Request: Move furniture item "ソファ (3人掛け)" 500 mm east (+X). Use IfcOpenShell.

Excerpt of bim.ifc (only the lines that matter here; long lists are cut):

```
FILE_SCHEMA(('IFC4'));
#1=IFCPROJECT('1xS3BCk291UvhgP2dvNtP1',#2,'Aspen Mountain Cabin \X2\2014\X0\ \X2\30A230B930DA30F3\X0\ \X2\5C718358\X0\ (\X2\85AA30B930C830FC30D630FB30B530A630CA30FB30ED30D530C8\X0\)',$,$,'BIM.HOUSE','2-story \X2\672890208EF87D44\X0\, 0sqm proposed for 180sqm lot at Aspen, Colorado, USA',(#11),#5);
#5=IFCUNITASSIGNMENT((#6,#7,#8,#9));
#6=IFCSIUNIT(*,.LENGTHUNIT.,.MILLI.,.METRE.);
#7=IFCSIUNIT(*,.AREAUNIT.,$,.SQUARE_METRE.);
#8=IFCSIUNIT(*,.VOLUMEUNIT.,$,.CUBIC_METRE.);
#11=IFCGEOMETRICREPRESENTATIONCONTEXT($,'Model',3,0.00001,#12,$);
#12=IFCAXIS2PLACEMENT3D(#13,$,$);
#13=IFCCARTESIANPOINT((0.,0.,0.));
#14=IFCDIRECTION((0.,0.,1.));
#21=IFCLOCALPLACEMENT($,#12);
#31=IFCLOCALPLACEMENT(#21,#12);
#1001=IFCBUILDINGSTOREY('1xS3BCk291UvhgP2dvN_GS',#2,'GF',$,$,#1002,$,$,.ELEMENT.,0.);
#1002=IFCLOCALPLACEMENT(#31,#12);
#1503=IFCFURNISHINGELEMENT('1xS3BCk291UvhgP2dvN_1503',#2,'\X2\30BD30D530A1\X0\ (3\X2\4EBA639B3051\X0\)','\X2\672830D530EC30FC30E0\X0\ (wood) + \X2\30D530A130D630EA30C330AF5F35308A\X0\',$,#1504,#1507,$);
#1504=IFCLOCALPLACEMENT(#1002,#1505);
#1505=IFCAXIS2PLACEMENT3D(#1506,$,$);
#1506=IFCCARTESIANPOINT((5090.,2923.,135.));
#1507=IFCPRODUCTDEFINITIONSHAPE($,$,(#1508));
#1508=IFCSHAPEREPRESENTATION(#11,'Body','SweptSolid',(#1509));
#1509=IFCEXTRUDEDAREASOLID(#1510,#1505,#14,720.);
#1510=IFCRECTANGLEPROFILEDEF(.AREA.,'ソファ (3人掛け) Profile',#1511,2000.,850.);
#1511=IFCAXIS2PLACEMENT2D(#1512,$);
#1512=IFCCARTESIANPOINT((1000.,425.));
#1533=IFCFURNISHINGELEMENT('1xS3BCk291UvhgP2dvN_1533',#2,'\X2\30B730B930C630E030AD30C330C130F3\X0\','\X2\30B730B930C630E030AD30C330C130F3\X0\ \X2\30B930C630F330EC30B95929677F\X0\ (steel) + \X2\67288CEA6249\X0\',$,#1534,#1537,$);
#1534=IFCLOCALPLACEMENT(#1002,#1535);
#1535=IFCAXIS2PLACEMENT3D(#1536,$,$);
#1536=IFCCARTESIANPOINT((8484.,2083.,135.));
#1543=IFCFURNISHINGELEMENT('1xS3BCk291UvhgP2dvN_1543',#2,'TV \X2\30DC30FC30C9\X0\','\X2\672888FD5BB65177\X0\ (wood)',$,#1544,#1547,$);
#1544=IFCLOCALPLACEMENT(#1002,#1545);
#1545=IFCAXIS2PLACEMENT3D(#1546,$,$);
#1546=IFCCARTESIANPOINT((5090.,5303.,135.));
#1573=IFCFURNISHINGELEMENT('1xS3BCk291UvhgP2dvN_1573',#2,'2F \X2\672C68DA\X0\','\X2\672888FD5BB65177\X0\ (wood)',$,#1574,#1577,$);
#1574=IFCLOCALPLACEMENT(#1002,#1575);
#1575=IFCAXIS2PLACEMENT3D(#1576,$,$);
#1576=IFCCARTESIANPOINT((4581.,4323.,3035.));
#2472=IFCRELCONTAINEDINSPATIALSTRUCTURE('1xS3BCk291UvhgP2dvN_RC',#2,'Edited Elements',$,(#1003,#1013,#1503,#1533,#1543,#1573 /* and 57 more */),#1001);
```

```python
import ifcopenshell
import ifcopenshell.api.geometry
import ifcopenshell.util.placement
import ifcopenshell.util.unit

model = ifcopenshell.open("bim.ifc")
unit_scale = ifcopenshell.util.unit.calculate_unit_scale(model)

item = model.by_guid("1xS3BCk291UvhgP2dvN_1503")
matrix = ifcopenshell.util.placement.get_local_placement(item.ObjectPlacement)
matrix[0, 3] += 0.5 / unit_scale
ifcopenshell.api.geometry.edit_object_placement(model, product=item, matrix=matrix, is_si=False)

print(ifcopenshell.util.placement.get_local_placement(item.ObjectPlacement).round(3) + 0.0)

model.write("bim_edited.ifc")
```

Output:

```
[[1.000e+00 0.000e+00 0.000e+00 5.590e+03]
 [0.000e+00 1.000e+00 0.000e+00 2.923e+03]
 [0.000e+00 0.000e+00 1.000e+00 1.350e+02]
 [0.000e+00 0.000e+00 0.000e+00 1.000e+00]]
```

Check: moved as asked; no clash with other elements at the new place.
